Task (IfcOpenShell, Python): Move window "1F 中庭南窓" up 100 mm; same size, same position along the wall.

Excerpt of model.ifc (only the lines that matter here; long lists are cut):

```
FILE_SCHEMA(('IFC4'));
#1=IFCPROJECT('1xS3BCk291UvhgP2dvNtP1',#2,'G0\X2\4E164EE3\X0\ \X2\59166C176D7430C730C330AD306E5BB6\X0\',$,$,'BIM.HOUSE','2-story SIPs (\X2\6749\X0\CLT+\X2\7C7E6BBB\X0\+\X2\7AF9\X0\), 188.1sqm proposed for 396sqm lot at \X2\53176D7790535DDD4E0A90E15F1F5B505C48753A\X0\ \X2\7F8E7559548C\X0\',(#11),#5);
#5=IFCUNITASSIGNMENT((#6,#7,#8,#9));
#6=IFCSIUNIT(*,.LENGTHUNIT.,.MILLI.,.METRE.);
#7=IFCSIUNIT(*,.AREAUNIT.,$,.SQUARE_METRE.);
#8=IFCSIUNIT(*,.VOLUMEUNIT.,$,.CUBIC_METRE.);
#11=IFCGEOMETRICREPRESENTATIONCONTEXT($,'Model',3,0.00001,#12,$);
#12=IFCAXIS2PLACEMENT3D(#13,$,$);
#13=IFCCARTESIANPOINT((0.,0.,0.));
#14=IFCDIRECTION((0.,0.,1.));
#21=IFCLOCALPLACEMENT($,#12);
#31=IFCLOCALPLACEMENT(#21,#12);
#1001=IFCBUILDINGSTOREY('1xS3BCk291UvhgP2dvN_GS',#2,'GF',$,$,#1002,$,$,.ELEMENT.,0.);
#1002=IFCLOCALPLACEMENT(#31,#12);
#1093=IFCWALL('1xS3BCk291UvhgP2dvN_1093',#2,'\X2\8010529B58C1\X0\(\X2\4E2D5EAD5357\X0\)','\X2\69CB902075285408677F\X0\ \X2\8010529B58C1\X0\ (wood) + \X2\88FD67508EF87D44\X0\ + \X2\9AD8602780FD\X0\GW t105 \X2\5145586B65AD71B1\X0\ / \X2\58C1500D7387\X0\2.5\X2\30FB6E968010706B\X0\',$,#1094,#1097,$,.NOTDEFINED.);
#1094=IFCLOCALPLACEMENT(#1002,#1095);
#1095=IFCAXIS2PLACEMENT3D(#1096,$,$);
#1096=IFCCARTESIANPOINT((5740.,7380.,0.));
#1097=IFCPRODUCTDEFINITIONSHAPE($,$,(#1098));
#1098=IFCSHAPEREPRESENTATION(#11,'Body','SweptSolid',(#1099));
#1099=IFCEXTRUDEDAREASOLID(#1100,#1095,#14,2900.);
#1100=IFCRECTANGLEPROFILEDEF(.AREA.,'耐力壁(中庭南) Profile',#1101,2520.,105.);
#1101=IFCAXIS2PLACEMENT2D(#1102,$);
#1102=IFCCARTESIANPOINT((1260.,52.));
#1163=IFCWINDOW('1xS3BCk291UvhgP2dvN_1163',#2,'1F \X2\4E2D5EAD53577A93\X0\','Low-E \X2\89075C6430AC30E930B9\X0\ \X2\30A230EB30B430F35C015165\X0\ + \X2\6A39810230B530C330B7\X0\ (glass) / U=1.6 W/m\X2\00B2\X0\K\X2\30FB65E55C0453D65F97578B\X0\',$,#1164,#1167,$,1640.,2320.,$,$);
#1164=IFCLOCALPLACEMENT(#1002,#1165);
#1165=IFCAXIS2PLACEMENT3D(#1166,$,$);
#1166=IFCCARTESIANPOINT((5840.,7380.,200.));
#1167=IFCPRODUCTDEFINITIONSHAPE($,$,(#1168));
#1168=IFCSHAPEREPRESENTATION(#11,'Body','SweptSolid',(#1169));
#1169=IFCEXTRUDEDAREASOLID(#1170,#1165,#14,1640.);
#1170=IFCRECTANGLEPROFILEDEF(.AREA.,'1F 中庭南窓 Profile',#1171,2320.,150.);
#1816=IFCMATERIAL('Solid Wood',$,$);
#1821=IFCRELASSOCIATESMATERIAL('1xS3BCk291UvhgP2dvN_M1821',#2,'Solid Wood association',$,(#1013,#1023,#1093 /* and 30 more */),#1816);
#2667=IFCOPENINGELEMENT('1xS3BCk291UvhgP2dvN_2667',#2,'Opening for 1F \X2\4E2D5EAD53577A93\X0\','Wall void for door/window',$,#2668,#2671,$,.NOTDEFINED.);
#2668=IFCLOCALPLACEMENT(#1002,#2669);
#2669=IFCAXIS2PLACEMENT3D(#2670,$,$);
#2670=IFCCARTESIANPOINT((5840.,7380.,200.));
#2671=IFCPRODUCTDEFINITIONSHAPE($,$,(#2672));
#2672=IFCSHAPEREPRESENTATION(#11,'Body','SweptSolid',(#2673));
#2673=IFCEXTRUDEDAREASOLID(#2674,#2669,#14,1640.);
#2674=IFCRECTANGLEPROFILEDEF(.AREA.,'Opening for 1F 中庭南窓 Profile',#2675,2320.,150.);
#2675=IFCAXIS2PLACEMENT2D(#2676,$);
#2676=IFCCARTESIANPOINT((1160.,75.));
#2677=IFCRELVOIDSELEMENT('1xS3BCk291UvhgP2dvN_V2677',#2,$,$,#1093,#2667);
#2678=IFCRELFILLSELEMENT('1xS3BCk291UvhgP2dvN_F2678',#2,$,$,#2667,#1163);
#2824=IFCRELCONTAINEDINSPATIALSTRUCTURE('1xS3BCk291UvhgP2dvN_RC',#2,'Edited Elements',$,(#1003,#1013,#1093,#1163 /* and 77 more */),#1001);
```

```python
import numpy as np
import ifcopenshell
import ifcopenshell.api.geometry
import ifcopenshell.util.placement
import ifcopenshell.util.unit

model = ifcopenshell.open("model.ifc")
unit_scale = ifcopenshell.util.unit.calculate_unit_scale(model)

window = model.by_guid("1xS3BCk291UvhgP2dvN_1163")
opening = window.FillsVoids[0].RelatingOpeningElement
dz = 0.1 / unit_scale

shift = np.array([0.0, 0.0, dz])
# The window is not placed relative to its opening, so move both.
for product in (opening, window):
    matrix = ifcopenshell.util.placement.get_local_placement(product.ObjectPlacement)
    matrix[:3, 3] += shift
    ifcopenshell.api.geometry.edit_object_placement(model, product=product, matrix=matrix, is_si=False)

print(f"moved by {dz * unit_scale:+.3f} m")

model.write("model_v2.ifc")
```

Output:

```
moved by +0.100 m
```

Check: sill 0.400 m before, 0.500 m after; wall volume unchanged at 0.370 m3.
